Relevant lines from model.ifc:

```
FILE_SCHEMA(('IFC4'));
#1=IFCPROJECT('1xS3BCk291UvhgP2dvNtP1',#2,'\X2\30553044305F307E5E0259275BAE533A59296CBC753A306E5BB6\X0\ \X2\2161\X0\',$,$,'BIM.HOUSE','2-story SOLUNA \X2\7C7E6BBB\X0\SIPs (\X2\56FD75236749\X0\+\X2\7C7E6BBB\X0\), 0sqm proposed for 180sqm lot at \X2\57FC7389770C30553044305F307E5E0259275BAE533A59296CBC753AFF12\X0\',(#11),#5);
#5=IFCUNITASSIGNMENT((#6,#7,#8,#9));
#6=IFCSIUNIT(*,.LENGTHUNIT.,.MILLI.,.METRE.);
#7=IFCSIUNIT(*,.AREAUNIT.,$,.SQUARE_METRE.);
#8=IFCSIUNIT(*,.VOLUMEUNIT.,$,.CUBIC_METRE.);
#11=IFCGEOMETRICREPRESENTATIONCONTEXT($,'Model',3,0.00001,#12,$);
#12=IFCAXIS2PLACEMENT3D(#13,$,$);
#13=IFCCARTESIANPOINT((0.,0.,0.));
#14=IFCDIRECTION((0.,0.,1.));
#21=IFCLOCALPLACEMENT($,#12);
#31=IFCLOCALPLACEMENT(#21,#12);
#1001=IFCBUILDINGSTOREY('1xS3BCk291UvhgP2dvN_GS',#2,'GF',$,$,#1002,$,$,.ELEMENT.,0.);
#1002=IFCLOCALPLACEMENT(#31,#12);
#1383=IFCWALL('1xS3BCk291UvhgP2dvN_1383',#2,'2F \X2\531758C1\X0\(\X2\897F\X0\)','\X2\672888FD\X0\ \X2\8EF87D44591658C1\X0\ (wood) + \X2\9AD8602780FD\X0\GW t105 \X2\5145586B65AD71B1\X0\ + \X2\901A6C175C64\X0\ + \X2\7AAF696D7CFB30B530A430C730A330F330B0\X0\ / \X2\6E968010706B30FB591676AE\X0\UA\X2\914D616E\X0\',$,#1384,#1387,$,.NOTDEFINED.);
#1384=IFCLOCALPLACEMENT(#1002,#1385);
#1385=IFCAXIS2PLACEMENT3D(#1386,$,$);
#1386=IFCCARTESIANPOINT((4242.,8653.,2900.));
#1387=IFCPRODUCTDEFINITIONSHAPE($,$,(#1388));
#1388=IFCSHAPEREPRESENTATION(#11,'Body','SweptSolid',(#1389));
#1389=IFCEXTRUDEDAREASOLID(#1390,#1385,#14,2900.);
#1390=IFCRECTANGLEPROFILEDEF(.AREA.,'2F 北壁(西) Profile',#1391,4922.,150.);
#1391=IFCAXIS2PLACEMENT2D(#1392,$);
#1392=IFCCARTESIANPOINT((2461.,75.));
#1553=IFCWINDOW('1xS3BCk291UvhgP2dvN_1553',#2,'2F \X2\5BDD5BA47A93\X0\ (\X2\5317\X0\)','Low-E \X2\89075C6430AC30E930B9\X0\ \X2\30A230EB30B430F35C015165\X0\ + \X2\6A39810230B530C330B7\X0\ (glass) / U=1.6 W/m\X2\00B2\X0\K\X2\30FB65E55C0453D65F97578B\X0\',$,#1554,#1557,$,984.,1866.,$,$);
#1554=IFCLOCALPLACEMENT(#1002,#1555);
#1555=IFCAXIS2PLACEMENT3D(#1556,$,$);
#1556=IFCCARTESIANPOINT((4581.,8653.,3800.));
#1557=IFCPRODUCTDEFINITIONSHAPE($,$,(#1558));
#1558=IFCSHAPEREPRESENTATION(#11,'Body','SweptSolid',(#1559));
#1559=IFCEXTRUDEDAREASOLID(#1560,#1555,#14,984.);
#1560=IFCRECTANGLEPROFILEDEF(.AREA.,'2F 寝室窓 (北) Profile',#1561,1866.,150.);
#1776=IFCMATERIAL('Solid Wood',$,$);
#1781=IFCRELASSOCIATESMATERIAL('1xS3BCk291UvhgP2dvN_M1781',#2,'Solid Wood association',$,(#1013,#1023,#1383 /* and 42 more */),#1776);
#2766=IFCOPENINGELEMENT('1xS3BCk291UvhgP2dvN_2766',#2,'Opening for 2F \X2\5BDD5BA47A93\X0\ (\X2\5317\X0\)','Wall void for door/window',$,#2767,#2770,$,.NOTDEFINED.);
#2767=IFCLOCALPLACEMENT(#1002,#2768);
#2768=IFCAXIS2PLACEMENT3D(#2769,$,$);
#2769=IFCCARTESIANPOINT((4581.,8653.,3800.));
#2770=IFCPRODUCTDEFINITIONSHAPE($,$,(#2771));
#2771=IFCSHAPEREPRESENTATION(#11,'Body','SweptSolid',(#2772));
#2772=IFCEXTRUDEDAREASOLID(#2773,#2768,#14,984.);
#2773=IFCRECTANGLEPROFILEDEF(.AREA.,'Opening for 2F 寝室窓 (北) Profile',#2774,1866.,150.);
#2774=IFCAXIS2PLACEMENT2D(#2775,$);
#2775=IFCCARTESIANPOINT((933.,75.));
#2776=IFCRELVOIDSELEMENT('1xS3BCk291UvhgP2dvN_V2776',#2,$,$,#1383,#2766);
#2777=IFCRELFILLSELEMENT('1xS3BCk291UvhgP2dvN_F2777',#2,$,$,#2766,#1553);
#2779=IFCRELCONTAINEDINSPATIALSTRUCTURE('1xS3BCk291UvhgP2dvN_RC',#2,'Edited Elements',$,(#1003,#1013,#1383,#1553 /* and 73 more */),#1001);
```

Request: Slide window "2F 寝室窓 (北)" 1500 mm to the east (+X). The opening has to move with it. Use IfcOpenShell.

```python
import ifcopenshell
import ifcopenshell.api.geometry
import ifcopenshell.util.placement

model = ifcopenshell.open("model.ifc")

window = model.by_id(1553)
opening = window.FillsVoids[0].RelatingOpeningElement
wall = opening.VoidsElements[0].RelatingBuildingElement

wall_matrix = ifcopenshell.util.placement.get_local_placement(wall.ObjectPlacement)
shift = wall_matrix[:3, 0] * 1500.0
before = ifcopenshell.util.placement.get_local_placement(window.ObjectPlacement)[:3, 3].copy()

# The window is not placed relative to its opening, so move both.
for product in (opening, window):
    matrix = ifcopenshell.util.placement.get_local_placement(product.ObjectPlacement)
    matrix[:3, 3] += shift
    ifcopenshell.api.geometry.edit_object_placement(model, product=product, matrix=matrix, is_si=False)

after = ifcopenshell.util.placement.get_local_placement(window.ObjectPlacement)[:3, 3]
print("window moved by", (after - before).round(3) + 0.0)

model.write("model_edited.ifc")
```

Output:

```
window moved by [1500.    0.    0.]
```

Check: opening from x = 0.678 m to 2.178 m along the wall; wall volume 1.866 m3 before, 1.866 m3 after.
